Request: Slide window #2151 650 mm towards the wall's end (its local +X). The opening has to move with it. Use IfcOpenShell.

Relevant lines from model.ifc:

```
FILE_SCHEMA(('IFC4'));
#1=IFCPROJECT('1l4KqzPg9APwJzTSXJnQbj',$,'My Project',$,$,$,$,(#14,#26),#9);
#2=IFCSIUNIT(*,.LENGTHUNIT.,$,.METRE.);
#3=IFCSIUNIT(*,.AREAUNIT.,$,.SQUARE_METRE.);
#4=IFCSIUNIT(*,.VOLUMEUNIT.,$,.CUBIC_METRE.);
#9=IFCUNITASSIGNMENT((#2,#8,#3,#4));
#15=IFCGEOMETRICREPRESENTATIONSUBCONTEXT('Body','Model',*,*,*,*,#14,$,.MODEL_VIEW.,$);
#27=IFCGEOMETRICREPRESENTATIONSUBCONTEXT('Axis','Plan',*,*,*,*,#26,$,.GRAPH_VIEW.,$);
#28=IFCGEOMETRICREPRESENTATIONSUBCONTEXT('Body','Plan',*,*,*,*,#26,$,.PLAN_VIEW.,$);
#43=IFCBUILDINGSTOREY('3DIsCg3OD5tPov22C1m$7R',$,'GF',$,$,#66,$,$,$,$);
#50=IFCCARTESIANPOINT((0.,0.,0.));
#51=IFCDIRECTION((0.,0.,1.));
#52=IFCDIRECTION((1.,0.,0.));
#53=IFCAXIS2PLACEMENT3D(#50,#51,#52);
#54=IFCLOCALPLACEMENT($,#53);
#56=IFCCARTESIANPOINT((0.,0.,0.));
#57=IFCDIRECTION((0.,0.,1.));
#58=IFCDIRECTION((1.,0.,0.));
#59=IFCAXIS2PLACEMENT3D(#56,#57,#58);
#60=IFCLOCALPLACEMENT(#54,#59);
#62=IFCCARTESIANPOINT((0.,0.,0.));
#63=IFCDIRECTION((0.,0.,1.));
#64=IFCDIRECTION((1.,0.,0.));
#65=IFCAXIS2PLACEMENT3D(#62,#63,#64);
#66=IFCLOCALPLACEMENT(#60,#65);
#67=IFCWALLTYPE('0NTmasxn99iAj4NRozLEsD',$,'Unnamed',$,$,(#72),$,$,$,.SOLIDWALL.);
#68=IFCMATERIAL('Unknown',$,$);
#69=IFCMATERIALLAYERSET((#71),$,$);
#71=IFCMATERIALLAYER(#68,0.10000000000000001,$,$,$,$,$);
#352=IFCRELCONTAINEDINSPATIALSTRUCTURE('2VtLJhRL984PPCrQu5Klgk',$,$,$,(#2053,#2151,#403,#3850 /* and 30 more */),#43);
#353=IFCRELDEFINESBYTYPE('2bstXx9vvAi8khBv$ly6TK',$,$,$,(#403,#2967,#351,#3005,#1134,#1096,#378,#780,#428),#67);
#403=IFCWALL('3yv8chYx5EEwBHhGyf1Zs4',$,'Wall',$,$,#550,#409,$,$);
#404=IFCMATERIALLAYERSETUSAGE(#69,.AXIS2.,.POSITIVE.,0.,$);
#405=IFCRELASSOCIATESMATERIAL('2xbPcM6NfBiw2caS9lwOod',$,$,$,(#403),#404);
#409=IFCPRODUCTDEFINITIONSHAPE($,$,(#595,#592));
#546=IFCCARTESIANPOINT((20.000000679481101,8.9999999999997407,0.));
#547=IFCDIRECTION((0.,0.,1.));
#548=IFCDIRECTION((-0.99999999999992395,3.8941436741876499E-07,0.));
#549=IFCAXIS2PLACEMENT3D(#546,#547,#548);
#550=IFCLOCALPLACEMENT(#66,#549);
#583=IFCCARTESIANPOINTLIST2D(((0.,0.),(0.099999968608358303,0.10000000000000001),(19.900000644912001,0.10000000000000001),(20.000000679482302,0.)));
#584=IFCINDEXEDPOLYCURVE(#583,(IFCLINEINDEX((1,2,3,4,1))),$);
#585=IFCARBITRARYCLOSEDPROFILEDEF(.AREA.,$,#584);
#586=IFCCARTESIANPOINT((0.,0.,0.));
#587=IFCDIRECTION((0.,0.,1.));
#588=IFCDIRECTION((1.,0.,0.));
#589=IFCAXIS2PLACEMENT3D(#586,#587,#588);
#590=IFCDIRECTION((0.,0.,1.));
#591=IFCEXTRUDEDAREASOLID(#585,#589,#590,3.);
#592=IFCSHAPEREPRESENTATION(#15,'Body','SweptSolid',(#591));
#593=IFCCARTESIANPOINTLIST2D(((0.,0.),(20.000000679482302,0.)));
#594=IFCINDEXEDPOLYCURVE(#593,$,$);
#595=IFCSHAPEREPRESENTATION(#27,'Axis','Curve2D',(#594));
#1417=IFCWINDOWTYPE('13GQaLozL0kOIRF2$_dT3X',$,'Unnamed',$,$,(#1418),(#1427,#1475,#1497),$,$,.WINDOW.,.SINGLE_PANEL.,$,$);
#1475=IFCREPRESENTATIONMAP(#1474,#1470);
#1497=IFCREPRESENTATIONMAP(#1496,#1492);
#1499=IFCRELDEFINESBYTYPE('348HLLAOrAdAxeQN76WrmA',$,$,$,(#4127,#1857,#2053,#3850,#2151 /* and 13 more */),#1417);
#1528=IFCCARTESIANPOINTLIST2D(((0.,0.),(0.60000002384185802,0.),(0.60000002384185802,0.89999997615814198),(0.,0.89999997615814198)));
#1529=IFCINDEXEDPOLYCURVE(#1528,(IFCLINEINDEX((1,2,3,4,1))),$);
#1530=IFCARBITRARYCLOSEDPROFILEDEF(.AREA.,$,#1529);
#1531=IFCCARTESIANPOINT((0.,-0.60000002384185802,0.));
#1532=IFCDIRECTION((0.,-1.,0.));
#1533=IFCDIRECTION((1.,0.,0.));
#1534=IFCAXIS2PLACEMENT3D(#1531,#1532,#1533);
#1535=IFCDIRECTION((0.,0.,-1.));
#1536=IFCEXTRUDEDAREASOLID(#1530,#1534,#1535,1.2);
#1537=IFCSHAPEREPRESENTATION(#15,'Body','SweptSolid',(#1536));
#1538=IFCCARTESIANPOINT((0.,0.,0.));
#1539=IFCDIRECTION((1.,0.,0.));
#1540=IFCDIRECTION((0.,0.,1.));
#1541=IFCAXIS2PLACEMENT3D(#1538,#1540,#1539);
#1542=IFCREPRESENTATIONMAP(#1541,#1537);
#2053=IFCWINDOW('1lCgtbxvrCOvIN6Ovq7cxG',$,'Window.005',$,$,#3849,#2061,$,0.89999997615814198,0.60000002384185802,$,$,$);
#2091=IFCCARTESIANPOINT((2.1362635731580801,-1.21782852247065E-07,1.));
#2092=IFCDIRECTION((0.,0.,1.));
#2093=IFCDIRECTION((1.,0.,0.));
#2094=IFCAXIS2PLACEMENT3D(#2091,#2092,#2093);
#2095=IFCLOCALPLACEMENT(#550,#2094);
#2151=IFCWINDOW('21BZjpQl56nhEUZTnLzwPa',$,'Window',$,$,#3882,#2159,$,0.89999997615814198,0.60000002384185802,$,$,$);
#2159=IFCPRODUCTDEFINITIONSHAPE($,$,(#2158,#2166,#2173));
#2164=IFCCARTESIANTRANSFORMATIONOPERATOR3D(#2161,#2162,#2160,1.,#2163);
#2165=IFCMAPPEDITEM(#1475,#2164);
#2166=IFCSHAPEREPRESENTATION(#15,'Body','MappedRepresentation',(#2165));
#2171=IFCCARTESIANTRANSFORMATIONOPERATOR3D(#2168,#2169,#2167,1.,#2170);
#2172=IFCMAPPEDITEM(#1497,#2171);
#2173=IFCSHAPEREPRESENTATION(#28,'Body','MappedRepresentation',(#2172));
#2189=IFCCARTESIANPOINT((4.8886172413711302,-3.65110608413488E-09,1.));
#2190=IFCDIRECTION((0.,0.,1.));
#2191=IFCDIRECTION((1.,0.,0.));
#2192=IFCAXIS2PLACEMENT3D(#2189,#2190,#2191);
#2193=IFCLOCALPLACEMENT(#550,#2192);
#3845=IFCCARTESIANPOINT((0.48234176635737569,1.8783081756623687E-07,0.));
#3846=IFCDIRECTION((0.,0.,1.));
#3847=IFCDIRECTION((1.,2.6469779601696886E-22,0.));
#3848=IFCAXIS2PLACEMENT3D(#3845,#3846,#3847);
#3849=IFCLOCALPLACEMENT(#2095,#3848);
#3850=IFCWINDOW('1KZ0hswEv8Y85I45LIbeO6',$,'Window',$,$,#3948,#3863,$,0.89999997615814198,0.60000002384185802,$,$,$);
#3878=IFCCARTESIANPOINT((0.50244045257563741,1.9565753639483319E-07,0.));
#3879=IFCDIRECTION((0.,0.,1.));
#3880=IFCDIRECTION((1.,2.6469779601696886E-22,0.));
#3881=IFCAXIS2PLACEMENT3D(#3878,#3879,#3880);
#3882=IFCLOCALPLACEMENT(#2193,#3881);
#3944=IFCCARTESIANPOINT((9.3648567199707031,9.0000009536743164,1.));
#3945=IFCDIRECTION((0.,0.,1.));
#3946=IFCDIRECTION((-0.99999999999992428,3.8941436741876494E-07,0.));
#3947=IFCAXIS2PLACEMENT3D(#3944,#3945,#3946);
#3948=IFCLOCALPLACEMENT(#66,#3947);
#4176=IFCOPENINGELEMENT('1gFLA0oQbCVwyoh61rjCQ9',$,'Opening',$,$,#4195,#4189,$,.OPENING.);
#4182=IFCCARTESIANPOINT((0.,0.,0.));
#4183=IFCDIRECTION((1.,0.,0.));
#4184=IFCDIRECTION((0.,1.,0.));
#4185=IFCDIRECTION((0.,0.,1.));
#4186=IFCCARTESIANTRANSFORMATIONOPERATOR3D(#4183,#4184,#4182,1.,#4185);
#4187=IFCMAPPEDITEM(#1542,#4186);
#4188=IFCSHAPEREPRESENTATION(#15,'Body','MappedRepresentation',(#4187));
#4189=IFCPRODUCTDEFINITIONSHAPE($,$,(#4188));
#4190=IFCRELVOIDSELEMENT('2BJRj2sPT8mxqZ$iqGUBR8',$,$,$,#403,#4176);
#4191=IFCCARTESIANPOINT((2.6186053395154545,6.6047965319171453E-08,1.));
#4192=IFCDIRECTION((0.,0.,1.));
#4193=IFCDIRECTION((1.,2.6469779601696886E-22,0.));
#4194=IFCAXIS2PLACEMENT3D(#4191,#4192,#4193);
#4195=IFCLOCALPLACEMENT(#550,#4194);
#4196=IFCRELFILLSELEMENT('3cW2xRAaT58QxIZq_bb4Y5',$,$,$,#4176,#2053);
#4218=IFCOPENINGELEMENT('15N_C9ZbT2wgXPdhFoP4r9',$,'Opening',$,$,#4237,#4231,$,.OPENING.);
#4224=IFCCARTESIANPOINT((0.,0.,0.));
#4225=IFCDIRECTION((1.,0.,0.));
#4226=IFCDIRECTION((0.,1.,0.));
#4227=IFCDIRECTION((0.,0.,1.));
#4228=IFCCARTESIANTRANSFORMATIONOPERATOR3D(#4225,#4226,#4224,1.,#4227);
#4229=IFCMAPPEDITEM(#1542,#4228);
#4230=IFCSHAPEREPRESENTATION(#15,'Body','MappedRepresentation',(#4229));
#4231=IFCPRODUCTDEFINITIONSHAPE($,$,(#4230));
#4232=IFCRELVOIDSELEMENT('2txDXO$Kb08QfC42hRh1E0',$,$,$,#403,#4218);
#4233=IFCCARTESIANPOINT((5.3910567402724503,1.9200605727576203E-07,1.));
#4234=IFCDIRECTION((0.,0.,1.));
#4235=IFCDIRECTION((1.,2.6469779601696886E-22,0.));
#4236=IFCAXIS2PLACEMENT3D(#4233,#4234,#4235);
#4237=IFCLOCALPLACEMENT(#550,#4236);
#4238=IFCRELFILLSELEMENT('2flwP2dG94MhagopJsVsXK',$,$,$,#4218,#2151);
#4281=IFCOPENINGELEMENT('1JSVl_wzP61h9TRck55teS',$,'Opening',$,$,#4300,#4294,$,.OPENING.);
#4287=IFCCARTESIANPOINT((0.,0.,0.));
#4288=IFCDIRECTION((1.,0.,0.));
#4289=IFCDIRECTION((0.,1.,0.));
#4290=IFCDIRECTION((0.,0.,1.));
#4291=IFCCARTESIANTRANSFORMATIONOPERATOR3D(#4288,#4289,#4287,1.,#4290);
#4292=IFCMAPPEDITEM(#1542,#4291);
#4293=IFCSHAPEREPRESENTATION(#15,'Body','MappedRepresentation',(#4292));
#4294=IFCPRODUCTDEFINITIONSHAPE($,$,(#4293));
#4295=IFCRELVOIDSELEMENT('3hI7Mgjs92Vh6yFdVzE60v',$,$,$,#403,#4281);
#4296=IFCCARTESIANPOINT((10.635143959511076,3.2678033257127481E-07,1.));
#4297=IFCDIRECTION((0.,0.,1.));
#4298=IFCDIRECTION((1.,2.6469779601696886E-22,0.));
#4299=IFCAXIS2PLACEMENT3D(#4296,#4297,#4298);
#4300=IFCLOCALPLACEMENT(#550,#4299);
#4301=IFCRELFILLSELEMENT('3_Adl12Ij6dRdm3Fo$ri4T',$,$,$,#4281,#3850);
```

```python
import ifcopenshell
import ifcopenshell.api.geometry
import ifcopenshell.util.placement
import ifcopenshell.util.unit

model = ifcopenshell.open("model.ifc")
unit_scale = ifcopenshell.util.unit.calculate_unit_scale(model)

window = model.by_id(2151)
opening = window.FillsVoids[0].RelatingOpeningElement
wall = opening.VoidsElements[0].RelatingBuildingElement

wall_matrix = ifcopenshell.util.placement.get_local_placement(wall.ObjectPlacement)
shift = wall_matrix[:3, 0] * 0.65 / unit_scale
before = ifcopenshell.util.placement.get_local_placement(window.ObjectPlacement)[:3, 3].copy()

# The window is not placed relative to its opening, so move both.
for product in (opening, window):
    matrix = ifcopenshell.util.placement.get_local_placement(product.ObjectPlacement)
    matrix[:3, 3] += shift
    ifcopenshell.api.geometry.edit_object_placement(model, product=product, matrix=matrix, is_si=False)

after = ifcopenshell.util.placement.get_local_placement(window.ObjectPlacement)[:3, 3]
print("window moved by", (after - before).round(3) + 0.0)

model.write("model_v2.ifc")
```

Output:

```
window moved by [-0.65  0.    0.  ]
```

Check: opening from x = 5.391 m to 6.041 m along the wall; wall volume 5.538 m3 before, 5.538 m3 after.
